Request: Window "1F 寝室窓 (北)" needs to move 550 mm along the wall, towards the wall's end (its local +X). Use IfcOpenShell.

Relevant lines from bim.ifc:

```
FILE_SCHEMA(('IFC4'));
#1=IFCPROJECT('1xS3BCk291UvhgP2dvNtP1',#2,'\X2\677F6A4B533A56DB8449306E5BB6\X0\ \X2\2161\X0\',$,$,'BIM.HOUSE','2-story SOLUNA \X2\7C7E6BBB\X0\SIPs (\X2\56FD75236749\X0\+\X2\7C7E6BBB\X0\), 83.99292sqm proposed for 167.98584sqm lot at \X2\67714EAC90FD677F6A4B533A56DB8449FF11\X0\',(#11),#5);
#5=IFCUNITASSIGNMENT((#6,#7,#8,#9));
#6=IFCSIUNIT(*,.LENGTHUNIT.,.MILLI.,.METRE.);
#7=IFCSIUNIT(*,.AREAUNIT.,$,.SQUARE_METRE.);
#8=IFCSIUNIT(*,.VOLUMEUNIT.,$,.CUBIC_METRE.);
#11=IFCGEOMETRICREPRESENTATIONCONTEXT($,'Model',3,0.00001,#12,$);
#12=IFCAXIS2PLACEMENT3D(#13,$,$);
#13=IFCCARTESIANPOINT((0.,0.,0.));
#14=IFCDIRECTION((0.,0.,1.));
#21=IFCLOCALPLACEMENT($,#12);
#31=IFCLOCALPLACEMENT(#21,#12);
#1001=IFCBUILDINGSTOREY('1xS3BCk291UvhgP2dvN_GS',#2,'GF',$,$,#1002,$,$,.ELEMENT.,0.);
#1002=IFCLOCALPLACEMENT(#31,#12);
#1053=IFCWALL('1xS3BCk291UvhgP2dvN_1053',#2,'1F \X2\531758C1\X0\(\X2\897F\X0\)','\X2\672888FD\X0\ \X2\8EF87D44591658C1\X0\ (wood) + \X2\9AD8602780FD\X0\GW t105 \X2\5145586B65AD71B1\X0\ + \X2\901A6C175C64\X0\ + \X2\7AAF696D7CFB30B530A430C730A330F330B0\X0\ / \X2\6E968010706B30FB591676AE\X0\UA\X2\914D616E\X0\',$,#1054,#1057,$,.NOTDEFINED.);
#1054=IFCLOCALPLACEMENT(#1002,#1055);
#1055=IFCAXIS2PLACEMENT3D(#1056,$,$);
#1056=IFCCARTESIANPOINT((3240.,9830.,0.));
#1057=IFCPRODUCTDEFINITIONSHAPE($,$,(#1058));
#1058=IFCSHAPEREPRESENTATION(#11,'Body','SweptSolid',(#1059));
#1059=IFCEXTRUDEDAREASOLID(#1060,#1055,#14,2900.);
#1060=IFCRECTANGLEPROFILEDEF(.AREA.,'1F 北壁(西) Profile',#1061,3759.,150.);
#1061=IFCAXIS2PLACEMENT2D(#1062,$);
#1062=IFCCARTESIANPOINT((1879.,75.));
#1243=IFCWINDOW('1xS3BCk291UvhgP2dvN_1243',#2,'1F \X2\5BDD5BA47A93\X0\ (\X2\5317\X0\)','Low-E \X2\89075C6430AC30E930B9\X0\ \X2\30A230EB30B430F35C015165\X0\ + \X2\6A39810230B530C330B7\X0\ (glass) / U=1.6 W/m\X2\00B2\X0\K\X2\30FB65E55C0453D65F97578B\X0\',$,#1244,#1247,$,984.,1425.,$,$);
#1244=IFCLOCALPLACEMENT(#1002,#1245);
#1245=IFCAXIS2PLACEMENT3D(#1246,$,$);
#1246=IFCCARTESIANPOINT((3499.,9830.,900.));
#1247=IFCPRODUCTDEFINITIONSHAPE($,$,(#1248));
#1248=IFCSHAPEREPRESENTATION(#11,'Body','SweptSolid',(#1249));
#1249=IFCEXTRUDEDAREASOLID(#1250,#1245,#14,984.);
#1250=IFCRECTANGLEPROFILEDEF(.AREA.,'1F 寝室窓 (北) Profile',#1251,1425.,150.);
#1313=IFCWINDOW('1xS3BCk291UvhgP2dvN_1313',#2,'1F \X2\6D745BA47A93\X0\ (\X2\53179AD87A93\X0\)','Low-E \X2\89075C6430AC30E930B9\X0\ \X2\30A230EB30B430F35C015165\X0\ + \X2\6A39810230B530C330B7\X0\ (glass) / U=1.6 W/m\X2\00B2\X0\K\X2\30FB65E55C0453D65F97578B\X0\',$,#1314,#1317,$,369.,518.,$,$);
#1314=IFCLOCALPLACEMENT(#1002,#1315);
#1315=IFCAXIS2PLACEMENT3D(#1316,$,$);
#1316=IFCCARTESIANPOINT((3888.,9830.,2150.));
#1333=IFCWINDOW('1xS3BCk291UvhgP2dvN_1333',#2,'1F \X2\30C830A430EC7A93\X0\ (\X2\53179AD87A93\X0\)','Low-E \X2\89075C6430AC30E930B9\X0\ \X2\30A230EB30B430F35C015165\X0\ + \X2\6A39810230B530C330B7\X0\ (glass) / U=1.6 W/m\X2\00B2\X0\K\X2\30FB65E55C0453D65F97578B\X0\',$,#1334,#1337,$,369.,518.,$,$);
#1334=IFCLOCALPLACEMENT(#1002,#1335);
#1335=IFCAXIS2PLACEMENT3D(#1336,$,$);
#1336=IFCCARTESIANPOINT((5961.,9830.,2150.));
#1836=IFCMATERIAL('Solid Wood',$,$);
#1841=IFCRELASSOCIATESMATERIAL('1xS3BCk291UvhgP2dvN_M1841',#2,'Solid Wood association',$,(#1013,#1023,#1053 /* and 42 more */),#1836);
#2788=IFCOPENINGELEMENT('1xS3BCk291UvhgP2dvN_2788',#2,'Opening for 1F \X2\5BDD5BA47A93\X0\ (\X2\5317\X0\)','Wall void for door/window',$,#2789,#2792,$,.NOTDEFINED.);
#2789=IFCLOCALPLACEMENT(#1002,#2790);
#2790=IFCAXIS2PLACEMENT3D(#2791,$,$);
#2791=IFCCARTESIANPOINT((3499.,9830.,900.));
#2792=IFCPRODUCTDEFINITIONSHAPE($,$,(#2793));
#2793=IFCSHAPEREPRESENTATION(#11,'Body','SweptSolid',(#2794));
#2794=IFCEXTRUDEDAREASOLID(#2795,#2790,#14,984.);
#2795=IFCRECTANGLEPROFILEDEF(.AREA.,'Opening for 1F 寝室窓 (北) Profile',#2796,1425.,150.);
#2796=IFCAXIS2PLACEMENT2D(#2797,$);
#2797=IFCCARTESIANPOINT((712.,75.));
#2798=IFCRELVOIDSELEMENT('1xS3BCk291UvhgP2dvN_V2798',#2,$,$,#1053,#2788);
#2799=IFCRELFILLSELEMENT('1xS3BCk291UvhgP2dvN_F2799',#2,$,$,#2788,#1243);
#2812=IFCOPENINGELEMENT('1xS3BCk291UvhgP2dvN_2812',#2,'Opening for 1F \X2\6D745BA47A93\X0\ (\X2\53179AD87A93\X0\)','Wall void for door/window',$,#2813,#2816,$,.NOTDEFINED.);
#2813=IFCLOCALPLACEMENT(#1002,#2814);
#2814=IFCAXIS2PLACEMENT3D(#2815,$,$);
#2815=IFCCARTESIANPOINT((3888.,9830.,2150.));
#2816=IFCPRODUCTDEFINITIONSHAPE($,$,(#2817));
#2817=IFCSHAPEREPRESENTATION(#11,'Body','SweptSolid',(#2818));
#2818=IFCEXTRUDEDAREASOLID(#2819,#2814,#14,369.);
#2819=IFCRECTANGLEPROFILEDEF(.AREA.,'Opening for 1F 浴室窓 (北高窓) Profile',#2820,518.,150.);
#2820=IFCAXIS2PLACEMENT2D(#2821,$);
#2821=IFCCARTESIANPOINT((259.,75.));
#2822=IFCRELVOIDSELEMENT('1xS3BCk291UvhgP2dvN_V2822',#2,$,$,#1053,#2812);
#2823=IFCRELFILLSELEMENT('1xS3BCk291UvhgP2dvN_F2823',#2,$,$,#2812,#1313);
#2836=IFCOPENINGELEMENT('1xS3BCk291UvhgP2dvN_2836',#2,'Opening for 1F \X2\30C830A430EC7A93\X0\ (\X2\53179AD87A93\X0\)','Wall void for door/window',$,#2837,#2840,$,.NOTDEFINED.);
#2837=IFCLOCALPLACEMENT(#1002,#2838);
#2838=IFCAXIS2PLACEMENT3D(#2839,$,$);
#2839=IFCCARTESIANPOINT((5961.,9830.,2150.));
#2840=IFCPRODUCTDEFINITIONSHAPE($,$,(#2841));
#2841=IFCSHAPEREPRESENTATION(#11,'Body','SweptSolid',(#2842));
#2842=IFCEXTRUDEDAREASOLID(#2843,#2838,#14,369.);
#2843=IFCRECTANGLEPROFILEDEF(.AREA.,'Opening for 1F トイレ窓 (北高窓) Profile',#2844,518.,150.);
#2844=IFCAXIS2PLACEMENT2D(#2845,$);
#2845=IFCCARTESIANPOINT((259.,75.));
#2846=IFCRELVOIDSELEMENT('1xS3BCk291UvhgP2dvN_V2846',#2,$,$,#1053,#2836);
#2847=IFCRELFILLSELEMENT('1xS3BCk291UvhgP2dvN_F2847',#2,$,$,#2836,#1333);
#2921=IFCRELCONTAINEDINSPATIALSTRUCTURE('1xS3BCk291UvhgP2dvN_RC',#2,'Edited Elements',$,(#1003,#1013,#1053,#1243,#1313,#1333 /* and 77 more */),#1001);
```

```python
import ifcopenshell
import ifcopenshell.api.geometry
import ifcopenshell.util.placement

model = ifcopenshell.open("bim.ifc")

window = model.by_guid("1xS3BCk291UvhgP2dvN_1243")
opening = window.FillsVoids[0].RelatingOpeningElement
wall = opening.VoidsElements[0].RelatingBuildingElement

wall_matrix = ifcopenshell.util.placement.get_local_placement(wall.ObjectPlacement)
shift = wall_matrix[:3, 0] * 550.0
before = ifcopenshell.util.placement.get_local_placement(window.ObjectPlacement)[:3, 3].copy()

# The window is not placed relative to its opening, so move both.
for product in (opening, window):
    matrix = ifcopenshell.util.placement.get_local_placement(product.ObjectPlacement)
    matrix[:3, 3] += shift
    ifcopenshell.api.geometry.edit_object_placement(model, product=product, matrix=matrix, is_si=False)

after = ifcopenshell.util.placement.get_local_placement(window.ObjectPlacement)[:3, 3]
print("window moved by", (after - before).round(3) + 0.0)

model.write("bim_rev.ifc")
```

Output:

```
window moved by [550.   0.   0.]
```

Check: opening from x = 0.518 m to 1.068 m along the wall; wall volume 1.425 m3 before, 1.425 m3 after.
